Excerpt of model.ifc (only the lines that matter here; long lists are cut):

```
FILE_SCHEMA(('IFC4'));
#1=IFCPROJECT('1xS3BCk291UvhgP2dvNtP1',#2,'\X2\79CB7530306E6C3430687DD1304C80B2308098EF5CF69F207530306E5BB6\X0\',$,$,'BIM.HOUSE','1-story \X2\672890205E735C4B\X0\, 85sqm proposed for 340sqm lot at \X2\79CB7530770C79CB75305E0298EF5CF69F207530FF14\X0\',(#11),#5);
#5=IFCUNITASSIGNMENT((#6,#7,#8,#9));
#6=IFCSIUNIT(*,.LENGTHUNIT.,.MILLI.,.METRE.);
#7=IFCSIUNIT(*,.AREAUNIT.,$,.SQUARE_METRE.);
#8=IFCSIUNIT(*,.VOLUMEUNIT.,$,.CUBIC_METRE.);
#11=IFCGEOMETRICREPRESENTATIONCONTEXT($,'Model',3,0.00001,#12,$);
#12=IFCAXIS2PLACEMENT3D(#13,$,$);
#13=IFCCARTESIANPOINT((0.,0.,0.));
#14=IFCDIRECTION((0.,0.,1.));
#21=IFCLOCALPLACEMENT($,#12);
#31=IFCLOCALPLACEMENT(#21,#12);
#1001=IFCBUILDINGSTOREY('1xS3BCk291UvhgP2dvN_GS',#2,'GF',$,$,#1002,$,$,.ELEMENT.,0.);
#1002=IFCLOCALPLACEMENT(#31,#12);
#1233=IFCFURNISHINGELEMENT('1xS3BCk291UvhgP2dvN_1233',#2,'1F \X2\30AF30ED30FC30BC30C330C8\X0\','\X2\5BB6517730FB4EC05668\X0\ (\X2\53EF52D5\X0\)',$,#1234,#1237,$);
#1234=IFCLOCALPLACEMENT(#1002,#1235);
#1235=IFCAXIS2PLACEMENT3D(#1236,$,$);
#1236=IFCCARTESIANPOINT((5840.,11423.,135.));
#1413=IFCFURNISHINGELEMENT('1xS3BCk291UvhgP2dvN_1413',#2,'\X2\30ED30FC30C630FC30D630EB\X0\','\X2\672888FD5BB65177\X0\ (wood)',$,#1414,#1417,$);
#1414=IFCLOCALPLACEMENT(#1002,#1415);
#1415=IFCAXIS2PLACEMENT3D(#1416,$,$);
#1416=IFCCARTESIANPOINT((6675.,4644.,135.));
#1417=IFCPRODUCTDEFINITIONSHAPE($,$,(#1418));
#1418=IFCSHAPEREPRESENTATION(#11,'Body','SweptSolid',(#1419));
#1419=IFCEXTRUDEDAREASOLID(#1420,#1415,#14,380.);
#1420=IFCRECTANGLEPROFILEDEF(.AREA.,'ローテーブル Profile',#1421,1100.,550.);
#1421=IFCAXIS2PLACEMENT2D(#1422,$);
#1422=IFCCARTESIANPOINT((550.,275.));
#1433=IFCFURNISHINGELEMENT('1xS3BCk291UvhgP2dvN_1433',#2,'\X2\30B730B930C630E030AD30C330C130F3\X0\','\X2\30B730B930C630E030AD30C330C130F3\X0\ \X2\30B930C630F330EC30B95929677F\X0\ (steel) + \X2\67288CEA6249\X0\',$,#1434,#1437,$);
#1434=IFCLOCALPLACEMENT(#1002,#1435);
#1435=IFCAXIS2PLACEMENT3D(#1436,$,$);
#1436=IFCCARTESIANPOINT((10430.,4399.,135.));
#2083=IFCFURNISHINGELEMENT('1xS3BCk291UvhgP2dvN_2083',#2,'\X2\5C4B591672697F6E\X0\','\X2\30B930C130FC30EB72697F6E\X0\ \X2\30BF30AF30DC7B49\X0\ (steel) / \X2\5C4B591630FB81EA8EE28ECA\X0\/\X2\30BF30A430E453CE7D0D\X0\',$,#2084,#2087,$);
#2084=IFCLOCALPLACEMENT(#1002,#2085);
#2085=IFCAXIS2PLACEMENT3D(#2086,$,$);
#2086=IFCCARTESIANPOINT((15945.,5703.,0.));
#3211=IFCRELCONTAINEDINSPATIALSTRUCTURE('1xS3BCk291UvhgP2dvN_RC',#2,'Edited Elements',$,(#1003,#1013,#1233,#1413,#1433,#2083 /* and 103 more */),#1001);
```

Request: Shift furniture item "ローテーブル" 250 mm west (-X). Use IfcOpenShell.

```python
import ifcopenshell
import ifcopenshell.api.geometry
import ifcopenshell.util.placement
import ifcopenshell.util.unit

model = ifcopenshell.open("model.ifc")
unit_scale = ifcopenshell.util.unit.calculate_unit_scale(model)

item = model.by_guid("1xS3BCk291UvhgP2dvN_1413")
matrix = ifcopenshell.util.placement.get_local_placement(item.ObjectPlacement)
matrix[0, 3] -= 0.25 / unit_scale
ifcopenshell.api.geometry.edit_object_placement(model, product=item, matrix=matrix, is_si=False)

print(ifcopenshell.util.placement.get_local_placement(item.ObjectPlacement).round(3) + 0.0)

model.write("model_rev.ifc")
```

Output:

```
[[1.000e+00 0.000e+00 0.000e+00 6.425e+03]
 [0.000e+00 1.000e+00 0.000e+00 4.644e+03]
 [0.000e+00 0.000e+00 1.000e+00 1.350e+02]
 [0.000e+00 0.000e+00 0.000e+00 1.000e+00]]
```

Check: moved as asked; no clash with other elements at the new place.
